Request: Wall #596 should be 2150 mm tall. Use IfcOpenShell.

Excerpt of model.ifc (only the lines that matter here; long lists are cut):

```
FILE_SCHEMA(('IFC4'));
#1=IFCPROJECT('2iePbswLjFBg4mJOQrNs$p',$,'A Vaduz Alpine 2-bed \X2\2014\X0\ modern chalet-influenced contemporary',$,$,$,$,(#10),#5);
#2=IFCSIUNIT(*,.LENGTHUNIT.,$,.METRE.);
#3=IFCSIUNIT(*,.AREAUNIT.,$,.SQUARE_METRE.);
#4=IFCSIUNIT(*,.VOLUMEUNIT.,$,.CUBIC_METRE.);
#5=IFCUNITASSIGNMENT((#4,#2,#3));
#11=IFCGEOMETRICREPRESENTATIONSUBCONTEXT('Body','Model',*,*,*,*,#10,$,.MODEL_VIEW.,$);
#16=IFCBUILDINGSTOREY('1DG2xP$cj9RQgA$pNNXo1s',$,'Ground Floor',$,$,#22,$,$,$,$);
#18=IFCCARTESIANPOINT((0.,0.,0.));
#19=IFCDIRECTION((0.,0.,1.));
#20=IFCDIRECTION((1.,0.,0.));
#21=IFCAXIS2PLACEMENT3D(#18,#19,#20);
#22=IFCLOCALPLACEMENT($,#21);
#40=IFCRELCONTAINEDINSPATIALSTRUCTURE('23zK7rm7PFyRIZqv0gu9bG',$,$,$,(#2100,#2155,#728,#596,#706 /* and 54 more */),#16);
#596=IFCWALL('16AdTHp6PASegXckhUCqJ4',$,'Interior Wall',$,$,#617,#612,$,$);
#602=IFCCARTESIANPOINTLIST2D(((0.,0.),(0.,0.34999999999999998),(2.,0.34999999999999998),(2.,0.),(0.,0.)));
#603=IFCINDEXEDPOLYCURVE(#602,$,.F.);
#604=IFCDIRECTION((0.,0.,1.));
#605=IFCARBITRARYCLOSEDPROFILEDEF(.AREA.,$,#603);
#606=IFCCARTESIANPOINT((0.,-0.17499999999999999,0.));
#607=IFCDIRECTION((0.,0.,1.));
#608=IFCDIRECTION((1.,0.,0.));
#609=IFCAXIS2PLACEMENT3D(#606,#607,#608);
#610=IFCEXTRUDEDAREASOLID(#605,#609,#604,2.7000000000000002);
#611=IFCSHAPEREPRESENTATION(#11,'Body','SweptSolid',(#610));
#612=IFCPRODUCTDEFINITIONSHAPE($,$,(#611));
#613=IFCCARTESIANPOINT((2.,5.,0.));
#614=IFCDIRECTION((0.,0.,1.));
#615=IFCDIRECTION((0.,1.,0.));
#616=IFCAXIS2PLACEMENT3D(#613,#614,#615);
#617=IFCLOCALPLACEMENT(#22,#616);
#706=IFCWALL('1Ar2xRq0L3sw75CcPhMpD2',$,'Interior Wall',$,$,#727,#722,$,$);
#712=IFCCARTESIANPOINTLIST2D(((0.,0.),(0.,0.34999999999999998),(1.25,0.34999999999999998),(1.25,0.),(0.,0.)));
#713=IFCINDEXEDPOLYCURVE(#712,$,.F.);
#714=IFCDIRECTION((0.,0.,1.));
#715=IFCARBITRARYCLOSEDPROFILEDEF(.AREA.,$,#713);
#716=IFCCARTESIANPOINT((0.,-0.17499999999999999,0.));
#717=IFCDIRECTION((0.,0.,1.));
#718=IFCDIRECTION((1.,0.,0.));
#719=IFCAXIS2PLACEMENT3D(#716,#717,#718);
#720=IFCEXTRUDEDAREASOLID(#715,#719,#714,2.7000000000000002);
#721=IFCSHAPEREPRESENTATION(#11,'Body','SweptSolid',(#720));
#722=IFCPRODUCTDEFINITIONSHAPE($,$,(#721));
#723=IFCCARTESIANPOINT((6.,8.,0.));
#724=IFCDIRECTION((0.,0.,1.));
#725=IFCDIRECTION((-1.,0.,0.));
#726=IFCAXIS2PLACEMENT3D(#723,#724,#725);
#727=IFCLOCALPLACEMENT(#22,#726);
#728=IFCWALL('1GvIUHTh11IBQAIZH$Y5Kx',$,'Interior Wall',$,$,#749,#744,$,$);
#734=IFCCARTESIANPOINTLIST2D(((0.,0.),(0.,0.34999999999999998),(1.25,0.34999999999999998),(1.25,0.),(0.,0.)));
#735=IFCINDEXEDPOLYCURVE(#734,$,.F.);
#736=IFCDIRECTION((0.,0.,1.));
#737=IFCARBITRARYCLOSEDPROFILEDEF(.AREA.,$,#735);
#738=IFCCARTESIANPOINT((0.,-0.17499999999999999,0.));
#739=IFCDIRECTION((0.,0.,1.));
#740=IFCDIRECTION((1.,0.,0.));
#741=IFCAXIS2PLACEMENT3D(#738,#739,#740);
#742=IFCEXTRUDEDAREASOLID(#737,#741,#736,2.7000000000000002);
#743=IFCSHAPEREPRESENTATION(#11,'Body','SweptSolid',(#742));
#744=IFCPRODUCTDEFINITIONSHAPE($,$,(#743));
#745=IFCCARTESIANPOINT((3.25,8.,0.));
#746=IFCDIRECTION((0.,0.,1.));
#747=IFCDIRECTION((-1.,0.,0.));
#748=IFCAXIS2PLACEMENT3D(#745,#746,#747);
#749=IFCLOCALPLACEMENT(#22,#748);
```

```python
import ifcopenshell
import ifcopenshell.geom
import ifcopenshell.util.representation
import ifcopenshell.util.shape
import ifcopenshell.util.unit

model = ifcopenshell.open("model.ifc")
unit_scale = ifcopenshell.util.unit.calculate_unit_scale(model)
settings = ifcopenshell.geom.settings()


def volume(element):
    """Net volume in cubic metres, openings subtracted."""
    shape = ifcopenshell.geom.create_shape(settings, element)
    return ifcopenshell.util.shape.get_volume(shape.geometry)


wall = model.by_id(596)
before = volume(wall)

body = ifcopenshell.util.representation.get_representation(wall, "Model", "Body")
solid = body.Items[0]
old_height = solid.Depth
solid.Depth = 2.15 / unit_scale
after = volume(wall)

print(f"height {old_height:g} -> {solid.Depth:g}, volume {before:.3f} -> {after:.3f} m3")

model.write("model_rev.ifc")
```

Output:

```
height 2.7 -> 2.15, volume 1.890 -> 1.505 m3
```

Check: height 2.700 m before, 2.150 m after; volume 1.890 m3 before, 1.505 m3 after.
